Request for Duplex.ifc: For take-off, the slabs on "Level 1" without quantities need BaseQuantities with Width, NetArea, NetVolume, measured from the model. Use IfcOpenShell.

First a look at what the model holds.

```python
import ifcopenshell
import ifcopenshell.util.element
import ifcopenshell.util.unit

model = ifcopenshell.open("Duplex.ifc")
print(model.schema)
for unit_type in ("LENGTHUNIT", "AREAUNIT", "VOLUMEUNIT"):
    print(unit_type, ifcopenshell.util.unit.calculate_unit_scale(model, unit_type))
storey = next(s for s in model.by_type("IfcBuildingStorey") if s.Name == "Level 1")
slabs = [e for e in ifcopenshell.util.element.get_decomposition(storey) if e.is_a("IfcSlab")]
for e in sorted(slabs, key=lambda e: e.id()):
    print(e.id(), e.is_a(), e.Name, list(ifcopenshell.util.element.get_psets(e, qtos_only=True)), sep=" | ")
```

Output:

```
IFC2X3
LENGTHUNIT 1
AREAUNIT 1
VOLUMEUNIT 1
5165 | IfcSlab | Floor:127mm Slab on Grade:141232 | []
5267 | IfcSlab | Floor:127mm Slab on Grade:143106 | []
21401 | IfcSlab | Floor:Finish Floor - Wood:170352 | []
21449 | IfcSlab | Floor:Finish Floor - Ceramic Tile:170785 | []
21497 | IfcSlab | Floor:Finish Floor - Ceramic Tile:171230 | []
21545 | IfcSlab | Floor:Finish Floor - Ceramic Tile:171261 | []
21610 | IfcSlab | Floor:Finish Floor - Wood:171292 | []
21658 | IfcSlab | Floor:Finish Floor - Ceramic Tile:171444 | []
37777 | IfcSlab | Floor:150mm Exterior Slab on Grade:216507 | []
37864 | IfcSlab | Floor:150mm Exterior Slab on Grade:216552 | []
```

```python
import ifcopenshell
import ifcopenshell.api.pset
import ifcopenshell.geom
import ifcopenshell.util.element
import ifcopenshell.util.shape
import ifcopenshell.util.unit

model = ifcopenshell.open("Duplex.ifc")
unit_scale = ifcopenshell.util.unit.calculate_unit_scale(model)
area_scale = ifcopenshell.util.unit.calculate_unit_scale(model, "AREAUNIT")
volume_scale = ifcopenshell.util.unit.calculate_unit_scale(model, "VOLUMEUNIT")
settings = ifcopenshell.geom.settings()

storey = next(s for s in model.by_type("IfcBuildingStorey") if s.Name == "Level 1")
slabs = [e for e in ifcopenshell.util.element.get_decomposition(storey) if e.is_a("IfcSlab")]

for e in sorted(slabs, key=lambda e: e.id()):
    if ifcopenshell.util.element.get_psets(e, qtos_only=True, should_inherit=False):
        continue
    # Geometry comes back in metres, in the element's own axes.
    shape = ifcopenshell.geom.create_shape(settings, e)
    values = {
        "Width": ifcopenshell.util.shape.get_z(shape.geometry) / unit_scale,
        "NetArea": ifcopenshell.util.shape.get_footprint_area(shape.geometry) / area_scale,
        "NetVolume": ifcopenshell.util.shape.get_volume(shape.geometry) / volume_scale,
    }
    qto = ifcopenshell.api.pset.add_qto(model, product=e, name="BaseQuantities")
    ifcopenshell.api.pset.edit_qto(model, qto=qto, properties=values)
    print(e.id(), {k: round(v, 3) for k, v in values.items()})

model.write("Duplex_v2.ifc")
```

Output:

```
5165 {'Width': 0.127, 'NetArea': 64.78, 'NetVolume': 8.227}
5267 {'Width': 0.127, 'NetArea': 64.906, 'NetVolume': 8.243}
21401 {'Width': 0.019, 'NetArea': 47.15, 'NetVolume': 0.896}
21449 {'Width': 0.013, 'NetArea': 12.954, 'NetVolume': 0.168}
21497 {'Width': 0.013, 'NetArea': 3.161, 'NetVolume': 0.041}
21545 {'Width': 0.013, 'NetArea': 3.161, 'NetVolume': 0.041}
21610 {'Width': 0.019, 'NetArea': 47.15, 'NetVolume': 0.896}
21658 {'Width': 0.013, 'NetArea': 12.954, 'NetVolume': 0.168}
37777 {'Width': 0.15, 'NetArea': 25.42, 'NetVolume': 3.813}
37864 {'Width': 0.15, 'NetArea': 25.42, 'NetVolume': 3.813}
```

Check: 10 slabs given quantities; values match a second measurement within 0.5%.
